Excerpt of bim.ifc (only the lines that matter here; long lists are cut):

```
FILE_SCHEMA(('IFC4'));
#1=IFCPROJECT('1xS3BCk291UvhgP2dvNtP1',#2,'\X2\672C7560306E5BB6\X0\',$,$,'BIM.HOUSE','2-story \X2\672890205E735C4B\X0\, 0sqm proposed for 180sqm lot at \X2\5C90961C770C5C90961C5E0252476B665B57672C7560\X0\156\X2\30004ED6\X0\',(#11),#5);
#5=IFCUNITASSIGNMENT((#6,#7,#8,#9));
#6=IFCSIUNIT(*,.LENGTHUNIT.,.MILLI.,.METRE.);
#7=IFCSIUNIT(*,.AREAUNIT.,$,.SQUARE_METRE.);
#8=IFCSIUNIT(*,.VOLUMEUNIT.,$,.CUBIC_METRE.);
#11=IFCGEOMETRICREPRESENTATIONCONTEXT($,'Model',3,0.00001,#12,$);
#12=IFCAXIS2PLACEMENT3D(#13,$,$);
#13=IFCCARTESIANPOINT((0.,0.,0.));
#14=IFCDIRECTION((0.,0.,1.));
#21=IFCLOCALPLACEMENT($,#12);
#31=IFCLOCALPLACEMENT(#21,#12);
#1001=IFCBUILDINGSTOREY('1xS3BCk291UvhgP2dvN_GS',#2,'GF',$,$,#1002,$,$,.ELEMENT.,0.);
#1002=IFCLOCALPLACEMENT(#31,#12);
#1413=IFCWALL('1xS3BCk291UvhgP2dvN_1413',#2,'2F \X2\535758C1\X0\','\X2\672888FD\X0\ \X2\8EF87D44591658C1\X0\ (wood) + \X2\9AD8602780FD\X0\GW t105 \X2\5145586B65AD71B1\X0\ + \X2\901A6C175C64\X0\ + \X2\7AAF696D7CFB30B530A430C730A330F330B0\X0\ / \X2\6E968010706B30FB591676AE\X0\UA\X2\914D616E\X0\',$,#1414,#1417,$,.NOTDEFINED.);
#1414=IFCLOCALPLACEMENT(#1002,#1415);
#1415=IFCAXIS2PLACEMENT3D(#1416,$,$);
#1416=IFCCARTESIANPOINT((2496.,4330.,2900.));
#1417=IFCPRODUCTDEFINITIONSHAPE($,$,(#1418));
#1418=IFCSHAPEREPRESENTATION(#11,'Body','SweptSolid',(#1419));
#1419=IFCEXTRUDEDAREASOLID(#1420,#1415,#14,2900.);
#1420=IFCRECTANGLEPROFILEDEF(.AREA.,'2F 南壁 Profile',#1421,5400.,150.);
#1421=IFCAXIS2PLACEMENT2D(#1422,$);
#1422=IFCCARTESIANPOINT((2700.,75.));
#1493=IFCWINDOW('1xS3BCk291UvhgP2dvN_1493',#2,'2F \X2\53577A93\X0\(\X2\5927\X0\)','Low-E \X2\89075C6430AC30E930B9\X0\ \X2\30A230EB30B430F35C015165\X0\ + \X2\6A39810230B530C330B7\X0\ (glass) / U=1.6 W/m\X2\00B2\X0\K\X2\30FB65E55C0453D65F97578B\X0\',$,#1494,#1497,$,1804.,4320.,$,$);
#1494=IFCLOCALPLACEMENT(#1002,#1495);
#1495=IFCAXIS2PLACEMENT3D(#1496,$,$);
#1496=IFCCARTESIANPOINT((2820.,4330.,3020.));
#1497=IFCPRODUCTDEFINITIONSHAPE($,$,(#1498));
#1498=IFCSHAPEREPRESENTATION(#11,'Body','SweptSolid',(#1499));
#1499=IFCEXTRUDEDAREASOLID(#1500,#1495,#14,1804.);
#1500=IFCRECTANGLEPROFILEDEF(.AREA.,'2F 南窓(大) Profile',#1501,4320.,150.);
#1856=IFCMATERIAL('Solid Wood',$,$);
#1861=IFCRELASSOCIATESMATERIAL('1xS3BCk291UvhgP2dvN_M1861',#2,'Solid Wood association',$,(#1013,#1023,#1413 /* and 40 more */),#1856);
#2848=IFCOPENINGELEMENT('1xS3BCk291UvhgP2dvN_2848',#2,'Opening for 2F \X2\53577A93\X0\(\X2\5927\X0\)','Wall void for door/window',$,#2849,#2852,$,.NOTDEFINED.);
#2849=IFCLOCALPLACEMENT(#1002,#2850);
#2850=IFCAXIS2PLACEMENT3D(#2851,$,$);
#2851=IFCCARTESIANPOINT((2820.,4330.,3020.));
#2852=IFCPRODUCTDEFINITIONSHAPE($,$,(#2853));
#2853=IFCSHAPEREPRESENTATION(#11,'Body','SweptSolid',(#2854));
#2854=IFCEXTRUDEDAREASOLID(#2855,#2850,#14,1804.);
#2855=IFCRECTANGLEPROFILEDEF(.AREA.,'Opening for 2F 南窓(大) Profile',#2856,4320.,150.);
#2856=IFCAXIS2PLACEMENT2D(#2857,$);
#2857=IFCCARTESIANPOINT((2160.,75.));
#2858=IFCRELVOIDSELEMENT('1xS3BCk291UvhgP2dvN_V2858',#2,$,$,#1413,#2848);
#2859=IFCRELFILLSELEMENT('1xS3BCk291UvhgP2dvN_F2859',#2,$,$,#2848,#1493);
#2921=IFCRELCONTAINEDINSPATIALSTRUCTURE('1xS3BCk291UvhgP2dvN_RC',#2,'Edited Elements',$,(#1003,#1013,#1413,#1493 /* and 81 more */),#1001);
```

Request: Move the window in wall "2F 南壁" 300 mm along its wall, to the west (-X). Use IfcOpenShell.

```python
import ifcopenshell
import ifcopenshell.api.geometry
import ifcopenshell.util.placement
import ifcopenshell.util.unit

model = ifcopenshell.open("bim.ifc")
unit_scale = ifcopenshell.util.unit.calculate_unit_scale(model)

window = model.by_guid("1xS3BCk291UvhgP2dvN_1493")
opening = window.FillsVoids[0].RelatingOpeningElement
wall = opening.VoidsElements[0].RelatingBuildingElement

wall_matrix = ifcopenshell.util.placement.get_local_placement(wall.ObjectPlacement)
shift = wall_matrix[:3, 0] * -0.3 / unit_scale
before = ifcopenshell.util.placement.get_local_placement(window.ObjectPlacement)[:3, 3].copy()

# The window is not placed relative to its opening, so move both.
for product in (opening, window):
    matrix = ifcopenshell.util.placement.get_local_placement(product.ObjectPlacement)
    matrix[:3, 3] += shift
    ifcopenshell.api.geometry.edit_object_placement(model, product=product, matrix=matrix, is_si=False)

after = ifcopenshell.util.placement.get_local_placement(window.ObjectPlacement)[:3, 3]
print("window moved by", (after - before).round(3) + 0.0)

model.write("bim_updated.ifc")
```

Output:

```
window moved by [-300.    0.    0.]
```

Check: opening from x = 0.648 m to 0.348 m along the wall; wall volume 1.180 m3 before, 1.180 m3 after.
